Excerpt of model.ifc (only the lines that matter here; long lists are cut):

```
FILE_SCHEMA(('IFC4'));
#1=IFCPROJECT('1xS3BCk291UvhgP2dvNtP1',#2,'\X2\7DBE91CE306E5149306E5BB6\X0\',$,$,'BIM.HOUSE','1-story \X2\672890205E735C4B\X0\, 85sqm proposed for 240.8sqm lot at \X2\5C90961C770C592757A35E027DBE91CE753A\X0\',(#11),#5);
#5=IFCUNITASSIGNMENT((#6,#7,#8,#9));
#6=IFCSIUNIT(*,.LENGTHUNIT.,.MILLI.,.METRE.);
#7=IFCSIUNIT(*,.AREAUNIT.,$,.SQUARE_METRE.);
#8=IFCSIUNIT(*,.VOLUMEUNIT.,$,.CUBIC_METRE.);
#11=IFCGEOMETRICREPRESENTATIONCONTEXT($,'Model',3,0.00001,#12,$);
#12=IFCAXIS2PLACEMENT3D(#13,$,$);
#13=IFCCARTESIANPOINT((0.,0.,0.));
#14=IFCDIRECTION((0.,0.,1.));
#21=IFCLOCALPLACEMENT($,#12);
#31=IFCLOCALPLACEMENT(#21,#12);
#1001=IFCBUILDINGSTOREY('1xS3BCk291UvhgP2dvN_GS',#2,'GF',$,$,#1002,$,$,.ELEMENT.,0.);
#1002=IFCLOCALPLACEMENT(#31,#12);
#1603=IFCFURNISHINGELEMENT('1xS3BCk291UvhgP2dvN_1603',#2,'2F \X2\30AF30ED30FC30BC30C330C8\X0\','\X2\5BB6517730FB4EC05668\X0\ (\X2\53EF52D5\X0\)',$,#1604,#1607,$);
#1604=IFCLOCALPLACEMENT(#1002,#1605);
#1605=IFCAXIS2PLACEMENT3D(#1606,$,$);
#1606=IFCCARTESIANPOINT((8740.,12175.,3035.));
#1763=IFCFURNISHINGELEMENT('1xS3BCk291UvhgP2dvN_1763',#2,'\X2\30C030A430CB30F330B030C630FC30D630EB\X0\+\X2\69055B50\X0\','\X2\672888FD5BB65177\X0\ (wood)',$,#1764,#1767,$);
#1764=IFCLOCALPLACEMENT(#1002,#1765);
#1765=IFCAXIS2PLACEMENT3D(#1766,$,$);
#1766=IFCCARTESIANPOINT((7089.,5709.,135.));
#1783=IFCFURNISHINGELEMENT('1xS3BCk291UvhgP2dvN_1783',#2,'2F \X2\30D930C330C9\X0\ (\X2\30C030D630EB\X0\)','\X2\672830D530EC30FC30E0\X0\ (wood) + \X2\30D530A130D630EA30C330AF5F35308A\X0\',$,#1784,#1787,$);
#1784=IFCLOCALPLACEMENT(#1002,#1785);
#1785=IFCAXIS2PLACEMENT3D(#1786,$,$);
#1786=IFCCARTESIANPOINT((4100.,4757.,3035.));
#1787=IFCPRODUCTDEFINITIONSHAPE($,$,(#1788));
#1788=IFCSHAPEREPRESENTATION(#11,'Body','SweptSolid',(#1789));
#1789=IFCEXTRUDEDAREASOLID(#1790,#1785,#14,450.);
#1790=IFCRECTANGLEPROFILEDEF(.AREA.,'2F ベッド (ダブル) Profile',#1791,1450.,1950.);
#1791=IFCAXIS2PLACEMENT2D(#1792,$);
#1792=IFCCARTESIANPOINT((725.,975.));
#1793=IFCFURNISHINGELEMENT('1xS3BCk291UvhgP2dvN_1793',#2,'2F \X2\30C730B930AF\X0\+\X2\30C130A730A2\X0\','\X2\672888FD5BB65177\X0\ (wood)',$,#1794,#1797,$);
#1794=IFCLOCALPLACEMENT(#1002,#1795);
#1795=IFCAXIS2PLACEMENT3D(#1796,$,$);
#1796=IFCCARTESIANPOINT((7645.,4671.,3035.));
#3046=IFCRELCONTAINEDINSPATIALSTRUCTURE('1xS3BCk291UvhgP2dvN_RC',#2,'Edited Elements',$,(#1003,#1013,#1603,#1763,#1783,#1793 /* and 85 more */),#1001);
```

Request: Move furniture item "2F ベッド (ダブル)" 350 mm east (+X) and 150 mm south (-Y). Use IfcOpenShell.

```python
import ifcopenshell
import ifcopenshell.api.geometry
import ifcopenshell.util.placement
import ifcopenshell.util.unit

model = ifcopenshell.open("model.ifc")
unit_scale = ifcopenshell.util.unit.calculate_unit_scale(model)

item = model.by_guid("1xS3BCk291UvhgP2dvN_1783")
matrix = ifcopenshell.util.placement.get_local_placement(item.ObjectPlacement)
matrix[0, 3] += 0.35 / unit_scale
matrix[1, 3] -= 0.15 / unit_scale
ifcopenshell.api.geometry.edit_object_placement(model, product=item, matrix=matrix, is_si=False)

print(ifcopenshell.util.placement.get_local_placement(item.ObjectPlacement).round(3) + 0.0)

model.write("model_v2.ifc")
```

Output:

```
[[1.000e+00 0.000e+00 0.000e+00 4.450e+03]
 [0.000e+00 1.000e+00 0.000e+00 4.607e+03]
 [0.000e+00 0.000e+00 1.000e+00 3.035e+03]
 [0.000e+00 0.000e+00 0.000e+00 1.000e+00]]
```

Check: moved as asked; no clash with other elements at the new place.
